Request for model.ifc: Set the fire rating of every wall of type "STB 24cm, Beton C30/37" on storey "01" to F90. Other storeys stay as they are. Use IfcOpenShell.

First a look at what the model holds.

```python
import ifcopenshell
import ifcopenshell.util.element

model = ifcopenshell.open("model.ifc")
print(model.schema)
storey = next(s for s in model.by_type("IfcBuildingStorey") if s.Name == "01")
walls = [e for e in ifcopenshell.util.element.get_decomposition(storey) if e.is_a("IfcWall")]
seen = {}
for e in walls:
    element_type = ifcopenshell.util.element.get_type(e)
    key = (element_type.Name if element_type != e and element_type else None, ifcopenshell.util.element.get_pset(e, "Pset_WallCommon", "FireRating"))
    seen[key] = seen.get(key, 0) + 1
for (name, value), count in sorted(seen.items(), key=str):
    print(count, "x", name, "|", value)
```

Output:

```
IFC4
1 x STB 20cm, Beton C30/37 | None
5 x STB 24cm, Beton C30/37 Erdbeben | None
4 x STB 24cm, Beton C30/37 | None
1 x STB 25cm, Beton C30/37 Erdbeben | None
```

```python
import ifcopenshell
import ifcopenshell.api.pset
import ifcopenshell.util.element

model = ifcopenshell.open("model.ifc")

storey = next(s for s in model.by_type("IfcBuildingStorey") if s.Name == "01")
walls = [e for e in ifcopenshell.util.element.get_decomposition(storey) if e.is_a("IfcWall")]

count = 0
for e in walls:
    element_type = ifcopenshell.util.element.get_type(e)
    if element_type in (None, e) or element_type.Name != "STB 24cm, Beton C30/37":
        continue
    # add_pset returns the element's existing set when there is one.
    pset = ifcopenshell.api.pset.add_pset(model, product=e, name="Pset_WallCommon")
    ifcopenshell.api.pset.edit_pset(model, pset=pset, properties={"FireRating": "F90"})
    count += 1

print(count, "walls updated")

model.write("model_edited.ifc")
```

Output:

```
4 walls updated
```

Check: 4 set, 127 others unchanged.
